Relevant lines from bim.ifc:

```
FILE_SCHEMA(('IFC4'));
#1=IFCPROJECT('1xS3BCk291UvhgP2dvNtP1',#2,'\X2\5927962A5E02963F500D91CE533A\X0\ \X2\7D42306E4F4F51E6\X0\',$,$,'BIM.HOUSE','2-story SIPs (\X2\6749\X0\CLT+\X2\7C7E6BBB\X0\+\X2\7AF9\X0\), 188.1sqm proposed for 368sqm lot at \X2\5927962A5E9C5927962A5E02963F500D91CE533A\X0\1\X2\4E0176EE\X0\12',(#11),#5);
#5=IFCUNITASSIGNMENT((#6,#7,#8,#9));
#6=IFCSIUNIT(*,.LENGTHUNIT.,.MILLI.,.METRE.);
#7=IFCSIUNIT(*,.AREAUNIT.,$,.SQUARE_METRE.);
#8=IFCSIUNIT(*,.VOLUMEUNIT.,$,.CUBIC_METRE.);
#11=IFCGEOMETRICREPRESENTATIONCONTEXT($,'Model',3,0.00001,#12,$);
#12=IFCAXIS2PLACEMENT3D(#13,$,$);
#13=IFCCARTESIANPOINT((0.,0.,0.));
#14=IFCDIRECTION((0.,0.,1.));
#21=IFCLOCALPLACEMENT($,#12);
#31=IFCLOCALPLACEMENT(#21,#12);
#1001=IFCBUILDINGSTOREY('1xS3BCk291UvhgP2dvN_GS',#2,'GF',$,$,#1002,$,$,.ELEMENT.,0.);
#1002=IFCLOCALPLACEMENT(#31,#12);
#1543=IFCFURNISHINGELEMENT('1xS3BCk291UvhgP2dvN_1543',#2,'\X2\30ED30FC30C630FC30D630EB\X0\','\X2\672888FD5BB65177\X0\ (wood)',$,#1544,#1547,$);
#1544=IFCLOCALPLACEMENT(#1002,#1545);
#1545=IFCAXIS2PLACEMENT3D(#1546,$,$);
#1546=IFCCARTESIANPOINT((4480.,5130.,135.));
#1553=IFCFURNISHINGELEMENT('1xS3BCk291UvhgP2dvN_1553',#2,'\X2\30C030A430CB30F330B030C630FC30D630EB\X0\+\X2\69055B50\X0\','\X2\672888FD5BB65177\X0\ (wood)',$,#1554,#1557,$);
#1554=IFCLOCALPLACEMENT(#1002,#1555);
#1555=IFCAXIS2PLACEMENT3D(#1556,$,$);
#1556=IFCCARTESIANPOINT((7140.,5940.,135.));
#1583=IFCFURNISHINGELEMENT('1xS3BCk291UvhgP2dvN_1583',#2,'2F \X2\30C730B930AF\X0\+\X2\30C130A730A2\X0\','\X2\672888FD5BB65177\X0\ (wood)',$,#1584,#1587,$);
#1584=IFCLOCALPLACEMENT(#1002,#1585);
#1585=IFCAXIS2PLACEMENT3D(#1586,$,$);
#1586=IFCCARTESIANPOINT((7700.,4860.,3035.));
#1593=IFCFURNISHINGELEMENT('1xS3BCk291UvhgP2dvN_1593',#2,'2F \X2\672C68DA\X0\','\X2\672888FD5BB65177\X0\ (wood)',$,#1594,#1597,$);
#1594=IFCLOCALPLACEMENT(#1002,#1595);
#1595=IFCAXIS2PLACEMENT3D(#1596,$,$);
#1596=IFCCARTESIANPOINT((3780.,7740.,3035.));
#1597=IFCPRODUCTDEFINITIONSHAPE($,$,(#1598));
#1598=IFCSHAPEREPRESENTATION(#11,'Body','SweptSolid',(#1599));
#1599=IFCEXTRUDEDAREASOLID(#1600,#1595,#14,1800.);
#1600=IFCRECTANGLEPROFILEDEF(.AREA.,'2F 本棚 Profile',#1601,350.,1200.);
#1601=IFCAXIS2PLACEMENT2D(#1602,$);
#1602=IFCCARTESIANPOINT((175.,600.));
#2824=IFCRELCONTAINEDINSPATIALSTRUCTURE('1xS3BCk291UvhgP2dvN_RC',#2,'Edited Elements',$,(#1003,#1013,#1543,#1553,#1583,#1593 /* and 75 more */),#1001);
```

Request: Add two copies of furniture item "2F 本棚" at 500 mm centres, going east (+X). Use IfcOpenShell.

```python
import numpy as np
import ifcopenshell
import ifcopenshell.api.geometry
import ifcopenshell.api.root
import ifcopenshell.util.element
import ifcopenshell.util.placement

model = ifcopenshell.open("bim.ifc")


def reuse_history(source, copy):
    """copy_class also copies each property set's owner history, people and application; keep the originals."""
    for rel in copy.IsDefinedBy:
        if rel.is_a("IfcRelDefinesByProperties") and (history := rel.RelatingPropertyDefinition.OwnerHistory):
            rel.RelatingPropertyDefinition.OwnerHistory = source.OwnerHistory
            ifcopenshell.util.element.remove_deep2(model, history)


source = model.by_id(1593)
base = ifcopenshell.util.placement.get_local_placement(source.ObjectPlacement)
step = np.array([1.0, 0.0, 0.0]) * 500.0

for i in range(1, 3):
    copy = ifcopenshell.api.root.copy_class(model, product=source)
    copy.Representation = ifcopenshell.util.element.copy_deep(
        model, source.Representation, exclude=["IfcGeometricRepresentationContext", "IfcRepresentationMap"]
    )
    reuse_history(source, copy)
    matrix = base.copy()
    matrix[:3, 3] += i * step
    print("added at", matrix[:3, 3].round(3) + 0.0)
    ifcopenshell.api.geometry.edit_object_placement(model, product=copy, matrix=matrix, is_si=False)

model.write("bim-out.ifc")
```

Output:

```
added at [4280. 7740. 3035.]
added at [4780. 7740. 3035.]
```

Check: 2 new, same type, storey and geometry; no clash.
